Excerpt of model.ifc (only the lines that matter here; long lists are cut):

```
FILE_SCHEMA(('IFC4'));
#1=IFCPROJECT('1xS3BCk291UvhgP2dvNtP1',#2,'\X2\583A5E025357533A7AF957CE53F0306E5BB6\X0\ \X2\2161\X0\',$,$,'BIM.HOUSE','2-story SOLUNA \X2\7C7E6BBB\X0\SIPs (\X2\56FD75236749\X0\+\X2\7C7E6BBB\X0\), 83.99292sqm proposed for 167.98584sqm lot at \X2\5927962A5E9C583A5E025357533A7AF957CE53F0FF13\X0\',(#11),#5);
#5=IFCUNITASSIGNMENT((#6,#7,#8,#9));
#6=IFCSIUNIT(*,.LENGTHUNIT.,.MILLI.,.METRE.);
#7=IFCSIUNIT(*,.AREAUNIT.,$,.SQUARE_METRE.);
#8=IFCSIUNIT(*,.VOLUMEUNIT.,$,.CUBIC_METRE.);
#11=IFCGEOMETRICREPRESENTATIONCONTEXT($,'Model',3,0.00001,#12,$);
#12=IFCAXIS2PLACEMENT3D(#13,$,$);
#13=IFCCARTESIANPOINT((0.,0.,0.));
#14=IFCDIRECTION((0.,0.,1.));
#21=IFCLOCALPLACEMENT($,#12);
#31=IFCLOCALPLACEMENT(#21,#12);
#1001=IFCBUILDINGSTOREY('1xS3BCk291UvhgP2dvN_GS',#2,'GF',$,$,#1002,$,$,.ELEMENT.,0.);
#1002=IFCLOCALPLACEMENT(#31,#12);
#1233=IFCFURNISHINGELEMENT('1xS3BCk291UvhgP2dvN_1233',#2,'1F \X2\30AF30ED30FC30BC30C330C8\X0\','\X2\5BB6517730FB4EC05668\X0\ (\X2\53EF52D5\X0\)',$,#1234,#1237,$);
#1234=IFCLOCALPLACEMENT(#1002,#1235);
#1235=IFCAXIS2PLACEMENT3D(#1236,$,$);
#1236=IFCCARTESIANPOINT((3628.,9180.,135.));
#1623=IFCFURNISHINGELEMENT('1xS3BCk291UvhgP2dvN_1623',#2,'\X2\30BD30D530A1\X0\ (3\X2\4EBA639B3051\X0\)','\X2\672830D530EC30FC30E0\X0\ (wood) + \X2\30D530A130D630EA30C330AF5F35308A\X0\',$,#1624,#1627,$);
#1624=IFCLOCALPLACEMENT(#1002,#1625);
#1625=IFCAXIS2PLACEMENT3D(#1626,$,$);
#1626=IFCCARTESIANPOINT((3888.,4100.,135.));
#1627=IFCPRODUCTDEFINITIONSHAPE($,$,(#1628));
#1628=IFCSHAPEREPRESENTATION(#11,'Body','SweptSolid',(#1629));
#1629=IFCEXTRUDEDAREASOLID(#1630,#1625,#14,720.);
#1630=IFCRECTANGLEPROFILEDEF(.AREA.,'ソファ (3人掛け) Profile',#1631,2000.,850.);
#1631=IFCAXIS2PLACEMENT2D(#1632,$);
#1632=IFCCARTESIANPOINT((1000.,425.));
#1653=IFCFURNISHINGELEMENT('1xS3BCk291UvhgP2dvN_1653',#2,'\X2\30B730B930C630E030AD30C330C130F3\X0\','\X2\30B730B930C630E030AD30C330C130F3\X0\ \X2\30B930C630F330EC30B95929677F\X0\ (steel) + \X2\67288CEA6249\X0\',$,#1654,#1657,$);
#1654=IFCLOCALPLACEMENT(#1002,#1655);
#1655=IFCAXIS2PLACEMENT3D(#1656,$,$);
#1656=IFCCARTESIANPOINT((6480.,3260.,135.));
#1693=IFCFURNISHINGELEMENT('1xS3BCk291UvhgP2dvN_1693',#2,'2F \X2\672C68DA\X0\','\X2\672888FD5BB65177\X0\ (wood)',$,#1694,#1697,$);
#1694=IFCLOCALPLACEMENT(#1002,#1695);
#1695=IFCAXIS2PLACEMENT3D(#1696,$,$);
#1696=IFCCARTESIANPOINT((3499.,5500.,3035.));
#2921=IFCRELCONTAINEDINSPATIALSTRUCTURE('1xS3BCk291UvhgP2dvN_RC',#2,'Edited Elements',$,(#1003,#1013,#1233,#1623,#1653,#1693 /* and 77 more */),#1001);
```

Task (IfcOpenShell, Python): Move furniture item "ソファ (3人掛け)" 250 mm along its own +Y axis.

```python
import ifcopenshell
import ifcopenshell.api.geometry
import ifcopenshell.util.placement
import ifcopenshell.util.unit

model = ifcopenshell.open("model.ifc")
unit_scale = ifcopenshell.util.unit.calculate_unit_scale(model)

item = model.by_id(1623)
matrix = ifcopenshell.util.placement.get_local_placement(item.ObjectPlacement)
matrix[:3, 3] += matrix[:3, 1] * 0.25 / unit_scale
ifcopenshell.api.geometry.edit_object_placement(model, product=item, matrix=matrix, is_si=False)

print(ifcopenshell.util.placement.get_local_placement(item.ObjectPlacement).round(3) + 0.0)

model.write("model-out.ifc")
```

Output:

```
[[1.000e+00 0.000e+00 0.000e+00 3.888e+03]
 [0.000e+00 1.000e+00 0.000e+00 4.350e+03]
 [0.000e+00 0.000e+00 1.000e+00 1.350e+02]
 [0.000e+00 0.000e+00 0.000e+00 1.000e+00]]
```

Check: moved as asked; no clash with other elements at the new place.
